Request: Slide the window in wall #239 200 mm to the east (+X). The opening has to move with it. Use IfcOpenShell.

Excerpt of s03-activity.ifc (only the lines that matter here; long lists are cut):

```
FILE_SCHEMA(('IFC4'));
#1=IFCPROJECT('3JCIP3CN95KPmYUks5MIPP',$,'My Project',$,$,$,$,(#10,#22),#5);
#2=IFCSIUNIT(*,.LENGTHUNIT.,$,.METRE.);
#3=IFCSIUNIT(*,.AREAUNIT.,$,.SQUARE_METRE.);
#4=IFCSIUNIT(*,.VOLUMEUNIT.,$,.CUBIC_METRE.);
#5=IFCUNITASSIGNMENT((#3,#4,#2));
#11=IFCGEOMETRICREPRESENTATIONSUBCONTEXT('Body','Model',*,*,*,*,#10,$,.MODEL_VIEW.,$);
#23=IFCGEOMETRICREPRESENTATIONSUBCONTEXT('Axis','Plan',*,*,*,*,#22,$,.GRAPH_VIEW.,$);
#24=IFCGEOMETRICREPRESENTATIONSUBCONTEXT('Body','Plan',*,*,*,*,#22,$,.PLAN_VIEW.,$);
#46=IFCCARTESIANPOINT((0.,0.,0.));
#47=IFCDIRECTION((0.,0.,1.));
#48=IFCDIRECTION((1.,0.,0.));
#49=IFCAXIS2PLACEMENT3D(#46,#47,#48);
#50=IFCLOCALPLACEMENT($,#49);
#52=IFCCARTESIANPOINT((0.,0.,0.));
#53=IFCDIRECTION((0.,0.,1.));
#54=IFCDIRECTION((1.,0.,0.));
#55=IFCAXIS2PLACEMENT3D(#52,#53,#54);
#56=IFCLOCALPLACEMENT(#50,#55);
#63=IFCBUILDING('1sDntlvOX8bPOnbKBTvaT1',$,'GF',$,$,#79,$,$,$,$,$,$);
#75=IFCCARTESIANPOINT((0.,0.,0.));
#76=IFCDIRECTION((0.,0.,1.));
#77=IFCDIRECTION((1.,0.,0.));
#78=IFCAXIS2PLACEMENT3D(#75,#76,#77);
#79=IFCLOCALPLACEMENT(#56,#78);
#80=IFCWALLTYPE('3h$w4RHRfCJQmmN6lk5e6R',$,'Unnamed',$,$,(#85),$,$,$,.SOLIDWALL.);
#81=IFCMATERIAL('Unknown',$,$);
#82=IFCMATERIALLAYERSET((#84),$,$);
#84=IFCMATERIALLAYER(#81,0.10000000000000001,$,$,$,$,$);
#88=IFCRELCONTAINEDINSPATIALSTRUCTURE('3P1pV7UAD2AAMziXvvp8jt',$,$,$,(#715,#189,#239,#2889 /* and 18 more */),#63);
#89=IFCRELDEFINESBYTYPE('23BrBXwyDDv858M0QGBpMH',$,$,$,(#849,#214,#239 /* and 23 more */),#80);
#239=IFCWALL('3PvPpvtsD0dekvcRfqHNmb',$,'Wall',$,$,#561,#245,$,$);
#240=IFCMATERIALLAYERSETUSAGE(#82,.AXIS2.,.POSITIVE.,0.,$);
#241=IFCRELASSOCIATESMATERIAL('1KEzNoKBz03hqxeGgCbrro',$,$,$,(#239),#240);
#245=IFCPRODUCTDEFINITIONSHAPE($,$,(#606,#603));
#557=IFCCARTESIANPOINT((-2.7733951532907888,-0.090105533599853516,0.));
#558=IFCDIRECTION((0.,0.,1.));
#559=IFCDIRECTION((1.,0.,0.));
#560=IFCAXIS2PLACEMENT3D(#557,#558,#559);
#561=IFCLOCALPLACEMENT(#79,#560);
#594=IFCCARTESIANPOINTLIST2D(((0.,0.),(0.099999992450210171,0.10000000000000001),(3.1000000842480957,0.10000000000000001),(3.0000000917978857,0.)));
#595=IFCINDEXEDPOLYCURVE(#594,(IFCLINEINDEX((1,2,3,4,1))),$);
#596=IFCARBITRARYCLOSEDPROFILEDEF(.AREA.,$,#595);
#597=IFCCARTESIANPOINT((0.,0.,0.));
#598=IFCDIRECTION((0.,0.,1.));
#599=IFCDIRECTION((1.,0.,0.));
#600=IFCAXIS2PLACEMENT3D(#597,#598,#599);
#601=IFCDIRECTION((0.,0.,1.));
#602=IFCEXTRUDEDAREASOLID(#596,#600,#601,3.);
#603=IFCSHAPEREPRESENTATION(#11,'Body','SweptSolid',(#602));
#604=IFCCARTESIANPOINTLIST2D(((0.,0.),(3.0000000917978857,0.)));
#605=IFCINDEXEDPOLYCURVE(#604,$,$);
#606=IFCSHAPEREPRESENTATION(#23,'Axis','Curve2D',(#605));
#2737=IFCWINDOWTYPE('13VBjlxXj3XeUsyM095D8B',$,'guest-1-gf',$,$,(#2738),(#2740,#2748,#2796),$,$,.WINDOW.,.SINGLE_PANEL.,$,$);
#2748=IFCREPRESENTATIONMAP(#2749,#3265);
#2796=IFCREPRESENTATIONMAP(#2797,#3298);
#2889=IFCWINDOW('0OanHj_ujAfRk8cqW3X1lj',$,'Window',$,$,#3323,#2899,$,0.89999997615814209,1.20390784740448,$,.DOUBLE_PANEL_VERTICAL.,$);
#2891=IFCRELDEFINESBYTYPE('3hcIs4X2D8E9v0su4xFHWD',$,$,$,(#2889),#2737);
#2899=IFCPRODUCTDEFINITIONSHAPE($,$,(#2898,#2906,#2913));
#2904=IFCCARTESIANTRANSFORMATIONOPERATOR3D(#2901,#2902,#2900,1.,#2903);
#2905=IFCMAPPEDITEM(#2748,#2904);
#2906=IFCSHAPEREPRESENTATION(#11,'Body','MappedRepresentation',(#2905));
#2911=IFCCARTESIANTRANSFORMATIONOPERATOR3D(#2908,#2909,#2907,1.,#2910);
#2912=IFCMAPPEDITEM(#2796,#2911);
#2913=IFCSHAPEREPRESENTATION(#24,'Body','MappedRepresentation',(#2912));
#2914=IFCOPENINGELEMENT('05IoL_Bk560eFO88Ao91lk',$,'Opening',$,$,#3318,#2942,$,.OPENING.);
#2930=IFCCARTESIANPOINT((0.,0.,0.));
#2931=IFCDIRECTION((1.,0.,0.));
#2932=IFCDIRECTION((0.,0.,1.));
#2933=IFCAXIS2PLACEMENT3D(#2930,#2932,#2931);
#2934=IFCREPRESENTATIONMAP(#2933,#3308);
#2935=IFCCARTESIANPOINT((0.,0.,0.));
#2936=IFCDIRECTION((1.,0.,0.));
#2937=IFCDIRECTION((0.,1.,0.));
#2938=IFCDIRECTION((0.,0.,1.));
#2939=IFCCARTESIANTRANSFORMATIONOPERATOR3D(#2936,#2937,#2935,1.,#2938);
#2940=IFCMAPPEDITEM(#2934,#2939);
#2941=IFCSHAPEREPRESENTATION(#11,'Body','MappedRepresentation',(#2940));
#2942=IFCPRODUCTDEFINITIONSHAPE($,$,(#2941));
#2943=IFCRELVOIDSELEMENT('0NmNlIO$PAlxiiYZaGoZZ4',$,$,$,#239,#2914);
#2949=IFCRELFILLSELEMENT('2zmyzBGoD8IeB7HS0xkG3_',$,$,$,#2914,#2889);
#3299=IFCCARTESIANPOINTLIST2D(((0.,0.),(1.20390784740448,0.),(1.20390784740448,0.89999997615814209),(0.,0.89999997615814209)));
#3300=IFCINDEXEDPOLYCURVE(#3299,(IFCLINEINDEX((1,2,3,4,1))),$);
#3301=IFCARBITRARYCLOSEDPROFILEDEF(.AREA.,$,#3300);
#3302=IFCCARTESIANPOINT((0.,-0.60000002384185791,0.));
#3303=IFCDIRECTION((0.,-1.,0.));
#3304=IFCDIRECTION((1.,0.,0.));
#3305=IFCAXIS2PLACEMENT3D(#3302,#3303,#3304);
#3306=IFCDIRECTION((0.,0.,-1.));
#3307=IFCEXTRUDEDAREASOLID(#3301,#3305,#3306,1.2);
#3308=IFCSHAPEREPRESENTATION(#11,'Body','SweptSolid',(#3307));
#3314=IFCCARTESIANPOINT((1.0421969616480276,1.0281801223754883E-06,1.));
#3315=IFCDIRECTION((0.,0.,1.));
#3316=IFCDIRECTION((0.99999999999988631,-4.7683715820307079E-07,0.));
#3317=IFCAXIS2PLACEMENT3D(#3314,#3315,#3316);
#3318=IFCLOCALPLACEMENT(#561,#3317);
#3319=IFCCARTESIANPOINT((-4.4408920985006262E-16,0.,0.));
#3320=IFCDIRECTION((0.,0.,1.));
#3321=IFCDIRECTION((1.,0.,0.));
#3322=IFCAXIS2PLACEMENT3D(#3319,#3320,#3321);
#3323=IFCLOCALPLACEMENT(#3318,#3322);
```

```python
import ifcopenshell
import ifcopenshell.api.geometry
import ifcopenshell.util.placement

model = ifcopenshell.open("s03-activity.ifc")

window = model.by_id(2889)
opening = window.FillsVoids[0].RelatingOpeningElement
wall = opening.VoidsElements[0].RelatingBuildingElement

wall_matrix = ifcopenshell.util.placement.get_local_placement(wall.ObjectPlacement)
shift = wall_matrix[:3, 0] * 0.2
before = ifcopenshell.util.placement.get_local_placement(window.ObjectPlacement)[:3, 3].copy()

# The window is placed relative to its opening, so it follows when the opening moves.
matrix = ifcopenshell.util.placement.get_local_placement(opening.ObjectPlacement)
matrix[:3, 3] += shift
ifcopenshell.api.geometry.edit_object_placement(
    model, product=opening, matrix=matrix, is_si=False, should_transform_children=True
)

after = ifcopenshell.util.placement.get_local_placement(window.ObjectPlacement)[:3, 3]
print("window moved by", (after - before).round(3) + 0.0)

model.write("s03-activity_edited.ifc")
```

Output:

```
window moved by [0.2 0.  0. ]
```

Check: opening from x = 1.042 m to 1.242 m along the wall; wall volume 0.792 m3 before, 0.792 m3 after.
